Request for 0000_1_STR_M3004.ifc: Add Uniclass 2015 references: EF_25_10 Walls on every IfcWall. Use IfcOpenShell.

First a look at what the model holds.

```python
import ifcopenshell

model = ifcopenshell.open("0000_1_STR_M3004.ifc")
print(model.schema)
print("classifications:", [c.Name for c in model.by_type("IfcClassification")])
for ifc_class in ("IfcDoor", "IfcRoof", "IfcStair", "IfcWall", "IfcWindow"):
    print(ifc_class, len(model.by_type(ifc_class)))
```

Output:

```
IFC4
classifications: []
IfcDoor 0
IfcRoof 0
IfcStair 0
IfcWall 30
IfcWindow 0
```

```python
import ifcopenshell
import ifcopenshell.api.classification

model = ifcopenshell.open("0000_1_STR_M3004.ifc")

system = ifcopenshell.api.classification.add_classification(model, classification="Uniclass 2015")

codes = {
    "IfcWall": ("EF_25_10", "Walls"),
}
for ifc_class, (code, name) in codes.items():
    products = model.by_type(ifc_class)
    ifcopenshell.api.classification.add_reference(
        model, products=products, classification=system, identification=code, name=name
    )
    print(code, len(products))

model.write("0000_1_STR_M3004-out.ifc")
```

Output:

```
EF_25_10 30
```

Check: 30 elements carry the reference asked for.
